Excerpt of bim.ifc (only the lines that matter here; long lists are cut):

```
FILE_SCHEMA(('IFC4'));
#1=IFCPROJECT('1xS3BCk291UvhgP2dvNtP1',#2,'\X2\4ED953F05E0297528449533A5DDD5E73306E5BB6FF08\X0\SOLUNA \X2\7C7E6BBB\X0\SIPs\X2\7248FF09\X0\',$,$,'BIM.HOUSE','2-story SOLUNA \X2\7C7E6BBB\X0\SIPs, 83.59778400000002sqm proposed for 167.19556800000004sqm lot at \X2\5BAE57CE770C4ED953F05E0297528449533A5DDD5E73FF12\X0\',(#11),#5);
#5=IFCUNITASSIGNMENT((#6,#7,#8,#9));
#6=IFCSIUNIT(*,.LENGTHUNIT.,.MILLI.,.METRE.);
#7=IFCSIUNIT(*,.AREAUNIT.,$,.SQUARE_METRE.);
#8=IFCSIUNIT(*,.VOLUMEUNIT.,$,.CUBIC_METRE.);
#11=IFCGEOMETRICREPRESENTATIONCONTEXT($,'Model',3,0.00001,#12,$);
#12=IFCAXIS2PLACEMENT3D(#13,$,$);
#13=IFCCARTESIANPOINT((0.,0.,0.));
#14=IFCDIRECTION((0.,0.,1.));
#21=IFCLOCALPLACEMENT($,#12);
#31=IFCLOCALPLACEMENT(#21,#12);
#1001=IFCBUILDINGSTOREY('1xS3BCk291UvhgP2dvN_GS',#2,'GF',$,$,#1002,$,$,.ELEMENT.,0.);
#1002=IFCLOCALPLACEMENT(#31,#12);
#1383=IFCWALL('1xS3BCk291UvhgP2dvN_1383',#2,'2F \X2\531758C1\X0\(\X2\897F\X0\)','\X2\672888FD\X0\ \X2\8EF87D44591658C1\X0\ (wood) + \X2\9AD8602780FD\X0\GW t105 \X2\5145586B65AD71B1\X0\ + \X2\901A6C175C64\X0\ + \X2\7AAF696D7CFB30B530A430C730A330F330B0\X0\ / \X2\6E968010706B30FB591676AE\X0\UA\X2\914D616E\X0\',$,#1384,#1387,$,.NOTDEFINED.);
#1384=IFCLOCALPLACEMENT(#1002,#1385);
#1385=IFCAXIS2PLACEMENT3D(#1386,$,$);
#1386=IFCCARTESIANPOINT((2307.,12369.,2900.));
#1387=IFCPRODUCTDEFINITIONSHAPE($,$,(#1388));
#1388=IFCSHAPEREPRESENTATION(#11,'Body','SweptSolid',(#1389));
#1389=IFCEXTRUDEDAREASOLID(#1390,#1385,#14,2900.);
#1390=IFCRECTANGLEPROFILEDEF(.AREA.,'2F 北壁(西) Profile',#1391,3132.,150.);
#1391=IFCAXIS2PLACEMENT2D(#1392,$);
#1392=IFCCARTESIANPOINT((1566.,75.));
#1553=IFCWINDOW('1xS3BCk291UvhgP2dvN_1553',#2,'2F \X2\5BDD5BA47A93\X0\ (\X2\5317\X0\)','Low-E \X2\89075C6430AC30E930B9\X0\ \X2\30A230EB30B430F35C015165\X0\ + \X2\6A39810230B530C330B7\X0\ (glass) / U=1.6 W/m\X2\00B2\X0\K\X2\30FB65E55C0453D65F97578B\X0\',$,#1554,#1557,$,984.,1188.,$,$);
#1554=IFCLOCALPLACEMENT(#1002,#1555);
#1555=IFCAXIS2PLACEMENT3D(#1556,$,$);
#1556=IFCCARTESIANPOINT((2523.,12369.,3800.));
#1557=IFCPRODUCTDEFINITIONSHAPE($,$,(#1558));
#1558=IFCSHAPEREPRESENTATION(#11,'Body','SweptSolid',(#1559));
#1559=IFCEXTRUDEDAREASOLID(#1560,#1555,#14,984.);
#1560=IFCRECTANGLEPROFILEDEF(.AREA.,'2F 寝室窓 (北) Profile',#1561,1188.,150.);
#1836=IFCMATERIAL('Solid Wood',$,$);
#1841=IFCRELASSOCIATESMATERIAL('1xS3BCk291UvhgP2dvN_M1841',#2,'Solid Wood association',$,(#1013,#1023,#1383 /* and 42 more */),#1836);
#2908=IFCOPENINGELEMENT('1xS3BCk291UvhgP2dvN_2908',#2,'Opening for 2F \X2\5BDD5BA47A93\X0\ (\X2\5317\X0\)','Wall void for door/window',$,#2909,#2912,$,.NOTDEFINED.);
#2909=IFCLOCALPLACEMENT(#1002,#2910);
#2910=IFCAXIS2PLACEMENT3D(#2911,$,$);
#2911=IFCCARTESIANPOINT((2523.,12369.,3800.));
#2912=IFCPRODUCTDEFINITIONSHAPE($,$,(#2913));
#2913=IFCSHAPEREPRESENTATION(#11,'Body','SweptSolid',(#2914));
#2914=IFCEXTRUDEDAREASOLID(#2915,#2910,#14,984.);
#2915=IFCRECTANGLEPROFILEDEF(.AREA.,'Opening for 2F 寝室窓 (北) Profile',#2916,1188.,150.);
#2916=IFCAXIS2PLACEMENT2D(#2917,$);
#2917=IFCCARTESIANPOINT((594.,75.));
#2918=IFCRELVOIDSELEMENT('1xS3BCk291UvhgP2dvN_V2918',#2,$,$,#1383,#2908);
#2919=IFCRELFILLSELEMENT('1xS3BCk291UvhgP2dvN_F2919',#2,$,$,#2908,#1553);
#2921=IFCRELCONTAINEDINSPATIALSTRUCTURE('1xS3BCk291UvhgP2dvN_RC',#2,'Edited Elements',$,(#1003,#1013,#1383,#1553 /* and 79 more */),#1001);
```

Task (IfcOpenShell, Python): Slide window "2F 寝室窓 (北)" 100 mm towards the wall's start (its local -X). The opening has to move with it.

```python
import ifcopenshell
import ifcopenshell.api.geometry
import ifcopenshell.util.placement
import ifcopenshell.util.unit

model = ifcopenshell.open("bim.ifc")
unit_scale = ifcopenshell.util.unit.calculate_unit_scale(model)

window = model.by_guid("1xS3BCk291UvhgP2dvN_1553")
opening = window.FillsVoids[0].RelatingOpeningElement
wall = opening.VoidsElements[0].RelatingBuildingElement

wall_matrix = ifcopenshell.util.placement.get_local_placement(wall.ObjectPlacement)
shift = wall_matrix[:3, 0] * -0.1 / unit_scale
before = ifcopenshell.util.placement.get_local_placement(window.ObjectPlacement)[:3, 3].copy()

# The window is not placed relative to its opening, so move both.
for product in (opening, window):
    matrix = ifcopenshell.util.placement.get_local_placement(product.ObjectPlacement)
    matrix[:3, 3] += shift
    ifcopenshell.api.geometry.edit_object_placement(model, product=product, matrix=matrix, is_si=False)

after = ifcopenshell.util.placement.get_local_placement(window.ObjectPlacement)[:3, 3]
print("window moved by", (after - before).round(3) + 0.0)

model.write("bim_v2.ifc")
```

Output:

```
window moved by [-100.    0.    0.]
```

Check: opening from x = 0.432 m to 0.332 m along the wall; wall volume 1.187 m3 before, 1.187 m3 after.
